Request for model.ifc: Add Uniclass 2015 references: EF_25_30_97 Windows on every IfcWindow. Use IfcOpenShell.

First a look at what the model holds.

```python
import ifcopenshell

model = ifcopenshell.open("model.ifc")
print(model.schema)
print("classifications:", [c.Name for c in model.by_type("IfcClassification")])
for ifc_class in ("IfcDoor", "IfcRoof", "IfcStair", "IfcWall", "IfcWindow"):
    print(ifc_class, len(model.by_type(ifc_class)))
```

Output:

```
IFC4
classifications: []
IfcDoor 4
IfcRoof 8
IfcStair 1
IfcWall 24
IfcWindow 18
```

```python
import ifcopenshell
import ifcopenshell.api.classification

model = ifcopenshell.open("model.ifc")

system = ifcopenshell.api.classification.add_classification(model, classification="Uniclass 2015")

codes = {
    "IfcWindow": ("EF_25_30_97", "Windows"),
}
for ifc_class, (code, name) in codes.items():
    products = model.by_type(ifc_class)
    ifcopenshell.api.classification.add_reference(
        model, products=products, classification=system, identification=code, name=name
    )
    print(code, len(products))

model.write("model_v2.ifc")
```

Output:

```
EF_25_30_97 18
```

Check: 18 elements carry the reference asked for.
